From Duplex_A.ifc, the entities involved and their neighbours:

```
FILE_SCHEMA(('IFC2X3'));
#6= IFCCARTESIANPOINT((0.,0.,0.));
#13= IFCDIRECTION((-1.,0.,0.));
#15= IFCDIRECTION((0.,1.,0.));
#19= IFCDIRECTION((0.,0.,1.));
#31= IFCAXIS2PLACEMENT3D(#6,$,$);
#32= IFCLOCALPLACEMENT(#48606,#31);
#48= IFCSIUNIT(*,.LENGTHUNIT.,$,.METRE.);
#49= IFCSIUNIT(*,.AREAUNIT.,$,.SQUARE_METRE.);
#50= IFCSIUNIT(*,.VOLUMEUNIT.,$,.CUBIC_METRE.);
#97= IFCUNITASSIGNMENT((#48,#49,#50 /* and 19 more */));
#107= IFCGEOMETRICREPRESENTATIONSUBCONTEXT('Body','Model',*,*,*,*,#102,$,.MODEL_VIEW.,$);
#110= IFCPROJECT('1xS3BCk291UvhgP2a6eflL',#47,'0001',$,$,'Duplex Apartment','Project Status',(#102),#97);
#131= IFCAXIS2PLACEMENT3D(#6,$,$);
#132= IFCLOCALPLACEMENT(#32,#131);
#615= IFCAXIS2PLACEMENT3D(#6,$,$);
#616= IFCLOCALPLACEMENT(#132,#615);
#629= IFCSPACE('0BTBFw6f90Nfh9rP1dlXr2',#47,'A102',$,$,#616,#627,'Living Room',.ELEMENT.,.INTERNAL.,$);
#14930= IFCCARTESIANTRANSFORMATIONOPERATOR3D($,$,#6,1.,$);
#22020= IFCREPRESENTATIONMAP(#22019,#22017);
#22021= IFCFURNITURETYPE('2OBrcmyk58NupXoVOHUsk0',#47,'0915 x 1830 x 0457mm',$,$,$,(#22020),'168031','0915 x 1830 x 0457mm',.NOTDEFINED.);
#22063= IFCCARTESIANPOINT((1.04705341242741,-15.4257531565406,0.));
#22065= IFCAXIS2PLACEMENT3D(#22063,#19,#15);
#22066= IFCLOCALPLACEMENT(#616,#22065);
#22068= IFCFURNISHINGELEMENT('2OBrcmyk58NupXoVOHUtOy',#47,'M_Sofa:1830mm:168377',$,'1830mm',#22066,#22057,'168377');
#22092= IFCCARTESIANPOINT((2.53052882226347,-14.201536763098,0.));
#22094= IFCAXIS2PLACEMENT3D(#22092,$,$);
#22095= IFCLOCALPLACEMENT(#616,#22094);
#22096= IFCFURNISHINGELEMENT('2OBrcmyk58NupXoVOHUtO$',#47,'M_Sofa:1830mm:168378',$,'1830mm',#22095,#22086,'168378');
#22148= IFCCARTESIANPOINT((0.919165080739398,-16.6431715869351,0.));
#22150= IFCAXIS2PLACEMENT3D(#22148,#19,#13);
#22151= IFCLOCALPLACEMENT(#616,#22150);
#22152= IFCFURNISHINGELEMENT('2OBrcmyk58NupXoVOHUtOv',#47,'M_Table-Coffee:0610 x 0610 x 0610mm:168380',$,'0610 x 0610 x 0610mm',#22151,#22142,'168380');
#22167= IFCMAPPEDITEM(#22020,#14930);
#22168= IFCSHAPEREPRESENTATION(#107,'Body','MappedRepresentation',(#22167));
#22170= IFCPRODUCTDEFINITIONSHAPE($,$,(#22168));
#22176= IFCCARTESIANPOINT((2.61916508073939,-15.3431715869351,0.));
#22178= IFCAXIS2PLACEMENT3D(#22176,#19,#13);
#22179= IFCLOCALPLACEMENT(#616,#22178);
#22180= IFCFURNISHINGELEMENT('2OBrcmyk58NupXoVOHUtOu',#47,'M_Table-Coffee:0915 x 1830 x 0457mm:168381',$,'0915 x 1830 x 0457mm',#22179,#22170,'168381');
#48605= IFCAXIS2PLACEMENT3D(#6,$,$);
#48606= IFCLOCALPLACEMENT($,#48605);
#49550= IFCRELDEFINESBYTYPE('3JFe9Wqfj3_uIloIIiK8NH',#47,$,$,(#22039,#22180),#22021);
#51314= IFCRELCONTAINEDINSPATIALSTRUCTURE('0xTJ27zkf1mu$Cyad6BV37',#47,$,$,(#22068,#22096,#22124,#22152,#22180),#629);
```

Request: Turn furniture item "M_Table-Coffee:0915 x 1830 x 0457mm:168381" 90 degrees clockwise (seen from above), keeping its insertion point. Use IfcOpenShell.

```python
import ifcopenshell
import ifcopenshell.api.geometry
import ifcopenshell.util.placement

model = ifcopenshell.open("Duplex_A.ifc")

item = model.by_guid("2OBrcmyk58NupXoVOHUtOu")
matrix = ifcopenshell.util.placement.get_local_placement(item.ObjectPlacement)
matrix = matrix @ ifcopenshell.util.placement.rotation(-90, "Z")
ifcopenshell.api.geometry.edit_object_placement(model, product=item, matrix=matrix, is_si=False)

print(ifcopenshell.util.placement.get_local_placement(item.ObjectPlacement).round(3) + 0.0)

model.write("Duplex_A_edited.ifc")
```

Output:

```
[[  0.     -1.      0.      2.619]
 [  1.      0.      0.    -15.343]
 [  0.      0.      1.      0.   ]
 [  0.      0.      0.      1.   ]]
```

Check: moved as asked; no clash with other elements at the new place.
